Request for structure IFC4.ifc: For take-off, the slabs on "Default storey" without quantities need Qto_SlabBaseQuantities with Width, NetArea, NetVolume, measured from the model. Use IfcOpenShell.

First a look at what the model holds.

```python
import ifcopenshell
import ifcopenshell.util.element
import ifcopenshell.util.unit

model = ifcopenshell.open("structure IFC4.ifc")
print(model.schema)
for unit_type in ("LENGTHUNIT", "AREAUNIT", "VOLUMEUNIT"):
    print(unit_type, ifcopenshell.util.unit.calculate_unit_scale(model, unit_type))
storey = next(s for s in model.by_type("IfcBuildingStorey") if s.Name == "Default storey")
slabs = [e for e in ifcopenshell.util.element.get_decomposition(storey) if e.is_a("IfcSlab")]
for e in sorted(slabs, key=lambda e: e.id()):
    print(e.id(), e.is_a(), e.Name, list(ifcopenshell.util.element.get_psets(e, qtos_only=True)), sep=" | ")
```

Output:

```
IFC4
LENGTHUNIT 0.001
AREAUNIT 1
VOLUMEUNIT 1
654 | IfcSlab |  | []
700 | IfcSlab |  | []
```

```python
import ifcopenshell
import ifcopenshell.api.pset
import ifcopenshell.geom
import ifcopenshell.util.element
import ifcopenshell.util.shape
import ifcopenshell.util.unit

model = ifcopenshell.open("structure IFC4.ifc")
unit_scale = ifcopenshell.util.unit.calculate_unit_scale(model)
area_scale = ifcopenshell.util.unit.calculate_unit_scale(model, "AREAUNIT")
volume_scale = ifcopenshell.util.unit.calculate_unit_scale(model, "VOLUMEUNIT")
settings = ifcopenshell.geom.settings()

storey = next(s for s in model.by_type("IfcBuildingStorey") if s.Name == "Default storey")
slabs = [e for e in ifcopenshell.util.element.get_decomposition(storey) if e.is_a("IfcSlab")]

for e in sorted(slabs, key=lambda e: e.id()):
    if ifcopenshell.util.element.get_psets(e, qtos_only=True, should_inherit=False):
        continue
    # Geometry comes back in metres, in the element's own axes.
    shape = ifcopenshell.geom.create_shape(settings, e)
    values = {
        "Width": ifcopenshell.util.shape.get_z(shape.geometry) / unit_scale,
        "NetArea": ifcopenshell.util.shape.get_footprint_area(shape.geometry) / area_scale,
        "NetVolume": ifcopenshell.util.shape.get_volume(shape.geometry) / volume_scale,
    }
    qto = ifcopenshell.api.pset.add_qto(model, product=e, name="Qto_SlabBaseQuantities")
    ifcopenshell.api.pset.edit_qto(model, qto=qto, properties=values)
    print(e.id(), {k: round(v, 3) for k, v in values.items()})

model.write("structure IFC4_rev.ifc")
```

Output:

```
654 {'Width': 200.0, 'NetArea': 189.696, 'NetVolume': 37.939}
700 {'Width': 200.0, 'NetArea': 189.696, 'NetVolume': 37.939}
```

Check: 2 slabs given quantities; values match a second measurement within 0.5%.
